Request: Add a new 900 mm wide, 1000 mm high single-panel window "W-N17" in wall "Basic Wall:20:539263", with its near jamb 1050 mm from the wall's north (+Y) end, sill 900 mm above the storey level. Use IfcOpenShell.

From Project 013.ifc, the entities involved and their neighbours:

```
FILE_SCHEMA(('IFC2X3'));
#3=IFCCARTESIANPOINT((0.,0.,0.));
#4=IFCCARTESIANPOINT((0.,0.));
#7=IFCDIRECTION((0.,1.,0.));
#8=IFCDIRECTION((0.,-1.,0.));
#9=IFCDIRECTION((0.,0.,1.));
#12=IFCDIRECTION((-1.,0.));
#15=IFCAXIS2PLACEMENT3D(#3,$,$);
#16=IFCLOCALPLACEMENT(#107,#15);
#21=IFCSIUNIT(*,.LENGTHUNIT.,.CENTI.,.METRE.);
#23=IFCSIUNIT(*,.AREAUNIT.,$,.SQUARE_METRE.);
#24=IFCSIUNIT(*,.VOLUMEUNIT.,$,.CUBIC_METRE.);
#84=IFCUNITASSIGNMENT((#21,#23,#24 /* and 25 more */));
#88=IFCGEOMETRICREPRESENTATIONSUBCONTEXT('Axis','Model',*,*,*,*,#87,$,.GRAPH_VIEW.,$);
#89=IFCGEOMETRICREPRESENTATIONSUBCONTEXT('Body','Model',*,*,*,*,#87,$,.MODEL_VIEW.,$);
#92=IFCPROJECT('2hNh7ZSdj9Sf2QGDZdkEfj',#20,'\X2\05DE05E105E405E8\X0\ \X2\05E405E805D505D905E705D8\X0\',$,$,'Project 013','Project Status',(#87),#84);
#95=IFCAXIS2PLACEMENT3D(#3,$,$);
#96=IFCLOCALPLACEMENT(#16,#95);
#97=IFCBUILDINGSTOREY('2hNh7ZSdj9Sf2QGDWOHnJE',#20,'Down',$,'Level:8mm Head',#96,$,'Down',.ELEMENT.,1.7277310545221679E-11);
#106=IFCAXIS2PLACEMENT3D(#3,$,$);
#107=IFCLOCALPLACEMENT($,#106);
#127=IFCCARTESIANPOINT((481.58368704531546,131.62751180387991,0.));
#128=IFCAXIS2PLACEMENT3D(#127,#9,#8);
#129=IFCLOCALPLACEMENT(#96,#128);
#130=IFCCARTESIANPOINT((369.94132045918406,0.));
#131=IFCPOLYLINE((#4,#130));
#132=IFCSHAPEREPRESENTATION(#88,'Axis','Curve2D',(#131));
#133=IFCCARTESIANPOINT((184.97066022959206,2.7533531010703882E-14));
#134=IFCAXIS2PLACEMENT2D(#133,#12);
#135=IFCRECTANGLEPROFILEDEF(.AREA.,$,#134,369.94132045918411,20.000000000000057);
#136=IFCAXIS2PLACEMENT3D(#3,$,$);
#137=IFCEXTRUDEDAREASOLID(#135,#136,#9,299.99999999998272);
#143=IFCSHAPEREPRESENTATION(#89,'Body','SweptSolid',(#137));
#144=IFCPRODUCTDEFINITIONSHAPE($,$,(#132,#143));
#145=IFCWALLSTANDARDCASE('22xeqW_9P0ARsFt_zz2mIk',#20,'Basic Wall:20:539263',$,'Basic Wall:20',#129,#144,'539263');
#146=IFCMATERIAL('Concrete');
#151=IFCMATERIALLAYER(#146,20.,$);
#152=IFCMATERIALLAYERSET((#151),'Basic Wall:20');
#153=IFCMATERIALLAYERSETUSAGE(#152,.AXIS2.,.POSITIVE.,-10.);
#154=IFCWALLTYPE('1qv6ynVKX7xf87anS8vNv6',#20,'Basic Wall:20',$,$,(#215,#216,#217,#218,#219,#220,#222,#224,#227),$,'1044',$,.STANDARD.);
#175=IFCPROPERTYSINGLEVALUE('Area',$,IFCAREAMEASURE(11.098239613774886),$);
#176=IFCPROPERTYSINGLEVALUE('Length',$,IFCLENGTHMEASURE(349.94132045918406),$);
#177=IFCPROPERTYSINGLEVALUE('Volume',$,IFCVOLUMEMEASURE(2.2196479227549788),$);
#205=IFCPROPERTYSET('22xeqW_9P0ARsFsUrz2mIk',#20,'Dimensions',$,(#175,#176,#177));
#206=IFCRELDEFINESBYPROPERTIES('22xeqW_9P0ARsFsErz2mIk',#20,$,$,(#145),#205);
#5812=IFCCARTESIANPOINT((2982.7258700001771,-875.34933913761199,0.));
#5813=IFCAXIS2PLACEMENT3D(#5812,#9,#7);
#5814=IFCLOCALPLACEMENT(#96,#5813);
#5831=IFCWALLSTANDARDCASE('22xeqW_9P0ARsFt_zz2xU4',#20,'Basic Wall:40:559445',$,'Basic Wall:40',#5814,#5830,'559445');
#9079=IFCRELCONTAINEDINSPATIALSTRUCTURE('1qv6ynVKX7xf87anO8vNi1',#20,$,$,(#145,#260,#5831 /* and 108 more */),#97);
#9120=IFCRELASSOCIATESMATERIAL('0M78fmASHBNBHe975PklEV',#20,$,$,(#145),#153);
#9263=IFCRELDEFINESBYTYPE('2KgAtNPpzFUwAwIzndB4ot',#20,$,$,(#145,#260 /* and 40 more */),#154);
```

```python
import numpy as np
import ifcopenshell
import ifcopenshell.api.feature
import ifcopenshell.api.geometry
import ifcopenshell.api.pset
import ifcopenshell.api.root
import ifcopenshell.api.spatial
import ifcopenshell.api.type
import ifcopenshell.geom
import ifcopenshell.util.element
import ifcopenshell.util.placement
import ifcopenshell.util.representation
import ifcopenshell.util.shape
import ifcopenshell.util.unit

model = ifcopenshell.open("Project 013.ifc")
unit_scale = ifcopenshell.util.unit.calculate_unit_scale(model)
area_scale = ifcopenshell.util.unit.calculate_unit_scale(model, "AREAUNIT")
volume_scale = ifcopenshell.util.unit.calculate_unit_scale(model, "VOLUMEUNIT")
settings = ifcopenshell.geom.settings()


def volume(element):
    """Net volume in cubic metres, openings subtracted."""
    shape = ifcopenshell.geom.create_shape(settings, element)
    return ifcopenshell.util.shape.get_volume(shape.geometry)


wall = model.by_guid("22xeqW_9P0ARsFt_zz2mIk")
storey = ifcopenshell.util.element.get_container(wall, ifc_class="IfcBuildingStorey")
context = ifcopenshell.util.representation.get_context(model, "Model", "Body", "MODEL_VIEW")
before = volume(wall)

width, height, from_end, sill = 0.9, 1, 1.05, 0.9  # metres

# The wall runs along its own X axis, and the end named is its -X end.
wall_shape = ifcopenshell.geom.create_shape(settings, wall)
x, y, z = ifcopenshell.util.shape.get_vertices(wall_shape.geometry).T
start = x.min() + from_end
face, thickness = float(y.min()), float(y.max() - y.min())
wall_matrix = ifcopenshell.util.placement.get_local_placement(wall.ObjectPlacement)
level = ifcopenshell.util.placement.get_local_placement(storey.ObjectPlacement)[2, 3]


def in_wall(x, y):
    """Placement at x, y metres in the wall's axes, at sill height."""
    matrix = wall_matrix.copy()
    matrix[:, 3] = wall_matrix @ np.array([x / unit_scale, y / unit_scale, 0.0, 1.0])
    matrix[2, 3] = level + sill / unit_scale
    return matrix


# Opening: a box that overshoots both wall faces by 50 mm.
opening = ifcopenshell.api.root.create_entity(model, ifc_class="IfcOpeningElement")
box = ifcopenshell.api.geometry.add_wall_representation(
    model, context=context, length=width, height=height, thickness=thickness + 0.1
)
ifcopenshell.api.geometry.assign_representation(model, product=opening, representation=box)
ifcopenshell.api.geometry.edit_object_placement(model, product=opening, matrix=in_wall(start, face - 0.05), is_si=False)
ifcopenshell.api.feature.add_feature(model, feature=opening, element=wall)

window = ifcopenshell.api.root.create_entity(model, ifc_class="IfcWindow", name="W-N17")
window.OverallWidth, window.OverallHeight = width / unit_scale, height / unit_scale
body = ifcopenshell.api.geometry.add_window_representation(
    model,
    context=context,
    overall_width=window.OverallWidth,
    overall_height=window.OverallHeight,
    partition_type="SINGLE_PANEL",
)
ifcopenshell.api.geometry.assign_representation(model, product=window, representation=body)
ifcopenshell.api.spatial.assign_container(model, products=[window], relating_structure=storey)
fills = ifcopenshell.api.feature.add_filling(model, opening=opening, element=window)
fills.OwnerHistory = window.OwnerHistory  # required in IFC2X3

# IFC2X3 keeps the operation on the window style.
style = ifcopenshell.api.root.create_entity(model, ifc_class="IfcWindowStyle", name="W-N17")
style.OperationType, style.ConstructionType = "SINGLE_PANEL", "NOTDEFINED"
style.ParameterTakesPrecedence = style.Sizeable = False
ifcopenshell.api.type.assign_type(model, related_objects=[window], relating_type=style)

# Centre the window in the wall's thickness.
ifcopenshell.api.geometry.edit_object_placement(model, product=window, matrix=in_wall(start, face), is_si=False)
window_shape = ifcopenshell.geom.create_shape(settings, window)
depth = ifcopenshell.util.shape.get_vertices(window_shape.geometry)[:, 1]
offset = face + thickness / 2 - (depth.min() + depth.max()) / 2
ifcopenshell.api.geometry.edit_object_placement(model, product=window, matrix=in_wall(start, offset), is_si=False)

after = volume(wall)

# Update the wall's stored quantities.
pset = model.by_id(ifcopenshell.util.element.get_pset(wall, "Dimensions", should_inherit=False)["id"])
ifcopenshell.api.pset.edit_pset(model, pset=pset, properties={
    "Area": model.create_entity("IfcAreaMeasure", after / thickness / area_scale),
    "Volume": model.create_entity("IfcVolumeMeasure", after / volume_scale),
})

print(f"wall volume {before:.3f} -> {after:.3f} m3")

model.write("Project 013_rev.ifc")
```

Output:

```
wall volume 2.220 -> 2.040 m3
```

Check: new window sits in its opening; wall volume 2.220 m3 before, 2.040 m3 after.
